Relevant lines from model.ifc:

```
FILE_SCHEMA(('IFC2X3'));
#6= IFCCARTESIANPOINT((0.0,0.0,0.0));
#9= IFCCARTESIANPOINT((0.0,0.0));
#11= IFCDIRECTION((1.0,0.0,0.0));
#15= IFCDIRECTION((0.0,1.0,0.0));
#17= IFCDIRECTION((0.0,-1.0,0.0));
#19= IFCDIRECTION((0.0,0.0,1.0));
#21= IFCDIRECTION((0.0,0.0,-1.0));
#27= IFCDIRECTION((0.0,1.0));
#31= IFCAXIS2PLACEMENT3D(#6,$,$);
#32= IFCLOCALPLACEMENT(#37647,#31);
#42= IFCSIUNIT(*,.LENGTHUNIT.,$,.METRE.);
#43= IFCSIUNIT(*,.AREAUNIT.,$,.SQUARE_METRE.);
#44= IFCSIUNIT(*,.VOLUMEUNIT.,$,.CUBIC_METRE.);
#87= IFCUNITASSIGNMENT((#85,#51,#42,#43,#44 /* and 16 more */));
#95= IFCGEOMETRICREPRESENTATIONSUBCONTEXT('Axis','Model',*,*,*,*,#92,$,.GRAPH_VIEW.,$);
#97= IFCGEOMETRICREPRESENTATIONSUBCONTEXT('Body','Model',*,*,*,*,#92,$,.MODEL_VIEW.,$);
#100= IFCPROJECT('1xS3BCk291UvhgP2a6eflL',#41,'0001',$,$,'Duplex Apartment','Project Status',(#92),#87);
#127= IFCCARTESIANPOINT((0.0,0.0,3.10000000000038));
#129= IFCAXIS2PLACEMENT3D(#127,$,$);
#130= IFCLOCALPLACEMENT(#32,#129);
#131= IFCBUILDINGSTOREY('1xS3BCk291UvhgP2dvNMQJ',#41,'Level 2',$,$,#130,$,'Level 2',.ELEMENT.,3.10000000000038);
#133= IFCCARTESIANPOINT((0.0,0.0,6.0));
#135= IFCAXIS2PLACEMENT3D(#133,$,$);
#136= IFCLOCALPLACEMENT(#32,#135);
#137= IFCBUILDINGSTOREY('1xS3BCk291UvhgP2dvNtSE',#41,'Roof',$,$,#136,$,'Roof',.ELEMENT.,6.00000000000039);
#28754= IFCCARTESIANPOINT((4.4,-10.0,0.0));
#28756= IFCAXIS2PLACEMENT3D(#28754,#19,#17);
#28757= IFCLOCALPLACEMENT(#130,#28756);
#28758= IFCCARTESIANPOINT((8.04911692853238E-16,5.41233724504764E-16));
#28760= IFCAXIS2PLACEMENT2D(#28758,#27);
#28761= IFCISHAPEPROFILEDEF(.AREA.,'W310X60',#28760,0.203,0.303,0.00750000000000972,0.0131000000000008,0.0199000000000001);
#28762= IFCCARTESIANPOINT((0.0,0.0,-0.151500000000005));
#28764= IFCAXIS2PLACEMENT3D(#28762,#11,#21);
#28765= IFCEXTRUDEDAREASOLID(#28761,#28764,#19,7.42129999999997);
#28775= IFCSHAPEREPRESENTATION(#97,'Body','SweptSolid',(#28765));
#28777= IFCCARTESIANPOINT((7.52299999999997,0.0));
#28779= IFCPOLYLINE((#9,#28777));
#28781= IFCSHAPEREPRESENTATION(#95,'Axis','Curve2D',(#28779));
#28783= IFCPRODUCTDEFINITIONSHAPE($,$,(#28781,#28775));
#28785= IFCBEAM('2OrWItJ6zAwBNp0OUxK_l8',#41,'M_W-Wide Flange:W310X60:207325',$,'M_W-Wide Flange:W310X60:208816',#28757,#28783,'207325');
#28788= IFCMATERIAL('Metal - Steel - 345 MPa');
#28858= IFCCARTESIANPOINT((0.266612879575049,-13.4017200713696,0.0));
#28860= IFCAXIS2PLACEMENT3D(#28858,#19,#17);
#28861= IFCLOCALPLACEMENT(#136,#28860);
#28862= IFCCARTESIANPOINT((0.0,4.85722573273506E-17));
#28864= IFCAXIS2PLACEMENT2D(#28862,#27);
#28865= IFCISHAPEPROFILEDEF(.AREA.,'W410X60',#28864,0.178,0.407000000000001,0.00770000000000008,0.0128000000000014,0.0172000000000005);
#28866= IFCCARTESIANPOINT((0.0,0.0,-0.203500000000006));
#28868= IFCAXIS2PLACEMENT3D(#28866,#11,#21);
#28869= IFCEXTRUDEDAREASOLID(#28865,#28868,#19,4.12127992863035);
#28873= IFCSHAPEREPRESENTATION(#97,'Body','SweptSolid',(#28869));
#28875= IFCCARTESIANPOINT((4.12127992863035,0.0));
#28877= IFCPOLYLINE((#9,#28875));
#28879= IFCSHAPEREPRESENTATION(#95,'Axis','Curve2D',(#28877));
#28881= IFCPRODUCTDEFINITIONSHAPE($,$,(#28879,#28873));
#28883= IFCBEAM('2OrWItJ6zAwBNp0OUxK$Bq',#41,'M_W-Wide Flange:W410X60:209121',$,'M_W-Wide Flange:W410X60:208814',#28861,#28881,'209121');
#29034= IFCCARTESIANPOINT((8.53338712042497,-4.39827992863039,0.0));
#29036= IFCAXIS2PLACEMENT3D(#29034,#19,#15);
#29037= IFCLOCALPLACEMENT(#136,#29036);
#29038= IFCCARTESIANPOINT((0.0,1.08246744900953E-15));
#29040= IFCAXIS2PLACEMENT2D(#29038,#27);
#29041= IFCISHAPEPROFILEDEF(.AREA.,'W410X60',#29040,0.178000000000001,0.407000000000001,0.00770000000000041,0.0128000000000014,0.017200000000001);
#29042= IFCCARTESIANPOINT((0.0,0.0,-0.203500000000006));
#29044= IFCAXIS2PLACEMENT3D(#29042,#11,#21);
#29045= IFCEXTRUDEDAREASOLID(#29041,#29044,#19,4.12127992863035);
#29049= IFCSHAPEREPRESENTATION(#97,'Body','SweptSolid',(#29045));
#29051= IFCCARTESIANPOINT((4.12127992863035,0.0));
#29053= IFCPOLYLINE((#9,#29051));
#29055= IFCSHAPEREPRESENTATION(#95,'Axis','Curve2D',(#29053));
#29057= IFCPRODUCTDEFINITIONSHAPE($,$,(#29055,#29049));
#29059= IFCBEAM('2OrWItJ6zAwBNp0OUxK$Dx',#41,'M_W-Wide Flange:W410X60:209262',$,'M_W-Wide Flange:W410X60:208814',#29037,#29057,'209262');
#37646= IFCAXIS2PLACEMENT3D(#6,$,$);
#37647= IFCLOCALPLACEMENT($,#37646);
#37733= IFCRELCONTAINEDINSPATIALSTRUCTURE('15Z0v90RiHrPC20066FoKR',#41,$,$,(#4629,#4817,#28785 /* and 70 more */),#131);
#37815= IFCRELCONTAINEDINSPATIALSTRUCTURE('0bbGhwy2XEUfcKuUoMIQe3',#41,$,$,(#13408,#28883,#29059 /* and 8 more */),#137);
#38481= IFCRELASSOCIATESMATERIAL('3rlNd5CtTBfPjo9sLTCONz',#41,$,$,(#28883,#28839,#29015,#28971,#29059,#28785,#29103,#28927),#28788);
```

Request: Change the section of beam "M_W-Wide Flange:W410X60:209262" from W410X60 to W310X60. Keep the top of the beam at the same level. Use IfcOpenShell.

```python
import ifcopenshell
import ifcopenshell.util.element
import ifcopenshell.util.representation

model = ifcopenshell.open("model.ifc")

member = model.by_guid("2OrWItJ6zAwBNp0OUxK$Dx")
source = next(p for p in model.by_type("IfcIShapeProfileDef") if p.ProfileName == "W310X60")

body = ifcopenshell.util.representation.get_representation(member, "Model", "Body")
solid = body.Items[0]
old_profile = solid.SweptArea

# Copy the section's sizes but keep this member's own profile position.
profile = ifcopenshell.util.element.copy(model, source)
# Profiles are centred, so shift by half the change in depth to hold the top.
shift = (old_profile.OverallDepth - profile.OverallDepth) / 2
x, y = old_profile.Position.Location.Coordinates
up = (-1.0, 0.0)  # upwards, in the solid's own plane
location = model.createIfcCartesianPoint((x + up[0] * shift, y + up[1] * shift))
profile.Position = model.createIfcAxis2Placement2D(location, old_profile.Position.RefDirection)
solid.SweptArea = profile
if not model.get_total_inverses(old_profile):
    ifcopenshell.util.element.remove_deep2(model, old_profile)
member.Name = member.Name.replace("W410X60", "W310X60")
member.ObjectType = member.ObjectType.replace("W410X60", "W310X60")

print(solid.SweptArea)

model.write("model_edited.ifc")
```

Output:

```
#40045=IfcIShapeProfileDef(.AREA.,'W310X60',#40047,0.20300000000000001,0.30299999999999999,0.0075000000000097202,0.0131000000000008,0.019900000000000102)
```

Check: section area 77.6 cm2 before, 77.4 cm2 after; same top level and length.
